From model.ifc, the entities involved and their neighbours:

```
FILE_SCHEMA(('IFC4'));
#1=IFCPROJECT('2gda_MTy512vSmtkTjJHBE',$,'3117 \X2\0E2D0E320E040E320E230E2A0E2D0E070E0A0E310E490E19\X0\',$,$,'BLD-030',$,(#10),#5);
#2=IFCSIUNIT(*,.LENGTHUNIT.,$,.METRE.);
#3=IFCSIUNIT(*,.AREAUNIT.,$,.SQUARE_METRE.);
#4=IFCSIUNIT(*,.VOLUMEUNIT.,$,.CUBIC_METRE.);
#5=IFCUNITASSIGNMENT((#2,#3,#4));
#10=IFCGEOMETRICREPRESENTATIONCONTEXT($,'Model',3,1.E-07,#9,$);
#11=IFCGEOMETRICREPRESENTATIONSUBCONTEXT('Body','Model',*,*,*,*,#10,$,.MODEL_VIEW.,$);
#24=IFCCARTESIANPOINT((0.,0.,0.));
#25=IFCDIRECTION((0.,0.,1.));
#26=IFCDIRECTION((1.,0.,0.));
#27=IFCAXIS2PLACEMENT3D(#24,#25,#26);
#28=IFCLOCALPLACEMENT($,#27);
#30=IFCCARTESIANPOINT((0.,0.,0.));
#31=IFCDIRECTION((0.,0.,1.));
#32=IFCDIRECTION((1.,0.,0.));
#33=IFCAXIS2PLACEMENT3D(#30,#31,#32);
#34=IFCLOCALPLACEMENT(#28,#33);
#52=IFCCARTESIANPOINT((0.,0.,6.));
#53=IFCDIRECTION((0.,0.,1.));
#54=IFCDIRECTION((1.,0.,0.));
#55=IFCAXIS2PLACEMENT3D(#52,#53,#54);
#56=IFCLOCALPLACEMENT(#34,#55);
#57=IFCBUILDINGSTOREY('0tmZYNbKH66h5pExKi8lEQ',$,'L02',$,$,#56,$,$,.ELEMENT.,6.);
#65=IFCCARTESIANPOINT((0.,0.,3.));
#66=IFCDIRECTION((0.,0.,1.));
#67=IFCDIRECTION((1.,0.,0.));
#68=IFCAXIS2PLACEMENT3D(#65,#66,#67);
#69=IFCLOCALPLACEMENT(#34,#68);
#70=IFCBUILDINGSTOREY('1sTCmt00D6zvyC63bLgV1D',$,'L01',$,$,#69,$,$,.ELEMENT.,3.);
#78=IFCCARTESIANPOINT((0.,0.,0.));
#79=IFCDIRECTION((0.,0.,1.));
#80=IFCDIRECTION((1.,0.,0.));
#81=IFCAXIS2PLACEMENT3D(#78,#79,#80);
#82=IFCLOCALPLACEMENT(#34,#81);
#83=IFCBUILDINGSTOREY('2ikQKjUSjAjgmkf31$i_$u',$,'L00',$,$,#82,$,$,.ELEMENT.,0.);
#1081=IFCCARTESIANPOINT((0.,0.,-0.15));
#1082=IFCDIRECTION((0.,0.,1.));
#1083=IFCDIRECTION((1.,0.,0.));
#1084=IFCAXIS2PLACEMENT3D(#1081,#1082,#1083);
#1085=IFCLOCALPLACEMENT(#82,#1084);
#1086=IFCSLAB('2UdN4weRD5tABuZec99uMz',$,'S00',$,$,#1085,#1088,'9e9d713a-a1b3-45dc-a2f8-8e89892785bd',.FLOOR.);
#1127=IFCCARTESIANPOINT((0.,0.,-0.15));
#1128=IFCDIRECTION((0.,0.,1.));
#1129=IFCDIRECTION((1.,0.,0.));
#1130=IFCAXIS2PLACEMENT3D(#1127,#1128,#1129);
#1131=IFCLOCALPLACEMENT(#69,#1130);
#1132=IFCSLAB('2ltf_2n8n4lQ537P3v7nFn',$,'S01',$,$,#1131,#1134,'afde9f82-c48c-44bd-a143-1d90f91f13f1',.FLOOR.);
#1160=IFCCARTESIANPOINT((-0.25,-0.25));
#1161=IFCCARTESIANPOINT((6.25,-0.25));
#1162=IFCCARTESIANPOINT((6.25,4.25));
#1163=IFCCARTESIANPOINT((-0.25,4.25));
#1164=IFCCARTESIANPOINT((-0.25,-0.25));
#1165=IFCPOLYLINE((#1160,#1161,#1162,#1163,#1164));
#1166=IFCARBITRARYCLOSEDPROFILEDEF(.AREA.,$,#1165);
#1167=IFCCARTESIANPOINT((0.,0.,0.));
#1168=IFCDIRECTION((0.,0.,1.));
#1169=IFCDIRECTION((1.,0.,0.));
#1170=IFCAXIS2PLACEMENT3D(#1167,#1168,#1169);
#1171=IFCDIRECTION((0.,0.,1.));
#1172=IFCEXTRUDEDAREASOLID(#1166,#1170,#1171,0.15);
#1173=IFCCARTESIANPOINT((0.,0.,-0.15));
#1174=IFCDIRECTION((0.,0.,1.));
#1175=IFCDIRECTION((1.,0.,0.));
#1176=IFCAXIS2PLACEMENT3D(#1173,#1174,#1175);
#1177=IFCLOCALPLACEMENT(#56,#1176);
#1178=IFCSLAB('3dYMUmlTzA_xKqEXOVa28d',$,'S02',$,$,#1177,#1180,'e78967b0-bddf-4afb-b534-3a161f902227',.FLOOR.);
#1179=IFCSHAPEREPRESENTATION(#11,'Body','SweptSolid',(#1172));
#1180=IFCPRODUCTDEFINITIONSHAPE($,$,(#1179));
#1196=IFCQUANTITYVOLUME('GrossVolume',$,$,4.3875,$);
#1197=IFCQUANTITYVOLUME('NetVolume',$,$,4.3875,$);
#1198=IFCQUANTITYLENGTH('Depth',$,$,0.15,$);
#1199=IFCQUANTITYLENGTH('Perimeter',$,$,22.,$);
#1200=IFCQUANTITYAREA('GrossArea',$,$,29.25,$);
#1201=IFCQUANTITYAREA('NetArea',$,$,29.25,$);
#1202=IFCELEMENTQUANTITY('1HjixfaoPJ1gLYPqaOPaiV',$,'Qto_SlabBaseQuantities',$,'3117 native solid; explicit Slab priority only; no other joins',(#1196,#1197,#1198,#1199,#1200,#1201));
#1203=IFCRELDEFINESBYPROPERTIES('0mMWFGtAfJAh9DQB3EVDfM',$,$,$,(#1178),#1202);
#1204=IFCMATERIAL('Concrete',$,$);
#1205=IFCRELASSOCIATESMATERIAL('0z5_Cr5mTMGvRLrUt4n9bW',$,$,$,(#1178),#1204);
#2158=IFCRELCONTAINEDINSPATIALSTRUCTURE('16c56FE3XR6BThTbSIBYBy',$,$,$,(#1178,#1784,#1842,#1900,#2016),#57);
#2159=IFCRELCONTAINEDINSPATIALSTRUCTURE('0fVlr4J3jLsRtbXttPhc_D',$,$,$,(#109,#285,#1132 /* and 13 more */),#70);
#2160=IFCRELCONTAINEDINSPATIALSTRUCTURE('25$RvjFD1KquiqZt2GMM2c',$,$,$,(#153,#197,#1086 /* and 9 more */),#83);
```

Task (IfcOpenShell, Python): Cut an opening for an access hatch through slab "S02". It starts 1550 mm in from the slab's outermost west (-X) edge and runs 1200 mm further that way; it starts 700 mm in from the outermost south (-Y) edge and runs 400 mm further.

```python
import numpy as np
import ifcopenshell
import ifcopenshell.api.feature
import ifcopenshell.api.geometry
import ifcopenshell.api.pset
import ifcopenshell.api.root
import ifcopenshell.geom
import ifcopenshell.util.element
import ifcopenshell.util.placement
import ifcopenshell.util.representation
import ifcopenshell.util.shape
import ifcopenshell.util.unit

model = ifcopenshell.open("model.ifc")
unit_scale = ifcopenshell.util.unit.calculate_unit_scale(model)
area_scale = ifcopenshell.util.unit.calculate_unit_scale(model, "AREAUNIT")
volume_scale = ifcopenshell.util.unit.calculate_unit_scale(model, "VOLUMEUNIT")
settings = ifcopenshell.geom.settings()


def volume(element):
    """Net volume in cubic metres, openings subtracted."""
    shape = ifcopenshell.geom.create_shape(settings, element)
    return ifcopenshell.util.shape.get_volume(shape.geometry)


slab = model.by_id(1178)
before = volume(slab)

# Extent in the slab's own axes, in metres. The edges named are its -X and -Y sides.
slab_shape = ifcopenshell.geom.create_shape(settings, slab)
vertices = ifcopenshell.util.shape.get_vertices(slab_shape.geometry)
x_min, y_min, bottom = vertices.min(axis=0)
top = vertices[:, 2].max()

opening = ifcopenshell.api.root.create_entity(model, ifc_class="IfcOpeningElement", name="Access hatch opening", predefined_type="OPENING")
context = ifcopenshell.util.representation.get_context(model, "Model", "Body", "MODEL_VIEW")
width, depth = 1.2, 0.4
outline = [(0.0, 0.0), (width, 0.0), (width, depth), (0.0, depth), (0.0, 0.0)]
# Overshoot both faces by 50 mm so the cut is clean.
shape = ifcopenshell.api.geometry.add_slab_representation(
    model, context=context, depth=top - bottom + 0.1, polyline=outline
)
ifcopenshell.api.geometry.assign_representation(model, product=opening, representation=shape)

matrix = ifcopenshell.util.placement.get_local_placement(slab.ObjectPlacement)
matrix[:, 3] = matrix @ np.append(np.array([x_min + 1.55, y_min + 0.7, bottom - 0.05]) / unit_scale, 1.0)
ifcopenshell.api.geometry.edit_object_placement(model, product=opening, matrix=matrix, is_si=False)
ifcopenshell.api.feature.add_feature(model, feature=opening, element=slab)

after = volume(slab)

# Update the slab's stored quantities.
qto = model.by_id(ifcopenshell.util.element.get_pset(slab, "Qto_SlabBaseQuantities", should_inherit=False)["id"])
ifcopenshell.api.pset.edit_qto(model, qto=qto, properties={
    "NetVolume": after / volume_scale,
    "NetArea": after / (top - bottom) / area_scale,
})

print(f"slab volume {before:.3f} -> {after:.3f} m3")

model.write("model_v2.ifc")
```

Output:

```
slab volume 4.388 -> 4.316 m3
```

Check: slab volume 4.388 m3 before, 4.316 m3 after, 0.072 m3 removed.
